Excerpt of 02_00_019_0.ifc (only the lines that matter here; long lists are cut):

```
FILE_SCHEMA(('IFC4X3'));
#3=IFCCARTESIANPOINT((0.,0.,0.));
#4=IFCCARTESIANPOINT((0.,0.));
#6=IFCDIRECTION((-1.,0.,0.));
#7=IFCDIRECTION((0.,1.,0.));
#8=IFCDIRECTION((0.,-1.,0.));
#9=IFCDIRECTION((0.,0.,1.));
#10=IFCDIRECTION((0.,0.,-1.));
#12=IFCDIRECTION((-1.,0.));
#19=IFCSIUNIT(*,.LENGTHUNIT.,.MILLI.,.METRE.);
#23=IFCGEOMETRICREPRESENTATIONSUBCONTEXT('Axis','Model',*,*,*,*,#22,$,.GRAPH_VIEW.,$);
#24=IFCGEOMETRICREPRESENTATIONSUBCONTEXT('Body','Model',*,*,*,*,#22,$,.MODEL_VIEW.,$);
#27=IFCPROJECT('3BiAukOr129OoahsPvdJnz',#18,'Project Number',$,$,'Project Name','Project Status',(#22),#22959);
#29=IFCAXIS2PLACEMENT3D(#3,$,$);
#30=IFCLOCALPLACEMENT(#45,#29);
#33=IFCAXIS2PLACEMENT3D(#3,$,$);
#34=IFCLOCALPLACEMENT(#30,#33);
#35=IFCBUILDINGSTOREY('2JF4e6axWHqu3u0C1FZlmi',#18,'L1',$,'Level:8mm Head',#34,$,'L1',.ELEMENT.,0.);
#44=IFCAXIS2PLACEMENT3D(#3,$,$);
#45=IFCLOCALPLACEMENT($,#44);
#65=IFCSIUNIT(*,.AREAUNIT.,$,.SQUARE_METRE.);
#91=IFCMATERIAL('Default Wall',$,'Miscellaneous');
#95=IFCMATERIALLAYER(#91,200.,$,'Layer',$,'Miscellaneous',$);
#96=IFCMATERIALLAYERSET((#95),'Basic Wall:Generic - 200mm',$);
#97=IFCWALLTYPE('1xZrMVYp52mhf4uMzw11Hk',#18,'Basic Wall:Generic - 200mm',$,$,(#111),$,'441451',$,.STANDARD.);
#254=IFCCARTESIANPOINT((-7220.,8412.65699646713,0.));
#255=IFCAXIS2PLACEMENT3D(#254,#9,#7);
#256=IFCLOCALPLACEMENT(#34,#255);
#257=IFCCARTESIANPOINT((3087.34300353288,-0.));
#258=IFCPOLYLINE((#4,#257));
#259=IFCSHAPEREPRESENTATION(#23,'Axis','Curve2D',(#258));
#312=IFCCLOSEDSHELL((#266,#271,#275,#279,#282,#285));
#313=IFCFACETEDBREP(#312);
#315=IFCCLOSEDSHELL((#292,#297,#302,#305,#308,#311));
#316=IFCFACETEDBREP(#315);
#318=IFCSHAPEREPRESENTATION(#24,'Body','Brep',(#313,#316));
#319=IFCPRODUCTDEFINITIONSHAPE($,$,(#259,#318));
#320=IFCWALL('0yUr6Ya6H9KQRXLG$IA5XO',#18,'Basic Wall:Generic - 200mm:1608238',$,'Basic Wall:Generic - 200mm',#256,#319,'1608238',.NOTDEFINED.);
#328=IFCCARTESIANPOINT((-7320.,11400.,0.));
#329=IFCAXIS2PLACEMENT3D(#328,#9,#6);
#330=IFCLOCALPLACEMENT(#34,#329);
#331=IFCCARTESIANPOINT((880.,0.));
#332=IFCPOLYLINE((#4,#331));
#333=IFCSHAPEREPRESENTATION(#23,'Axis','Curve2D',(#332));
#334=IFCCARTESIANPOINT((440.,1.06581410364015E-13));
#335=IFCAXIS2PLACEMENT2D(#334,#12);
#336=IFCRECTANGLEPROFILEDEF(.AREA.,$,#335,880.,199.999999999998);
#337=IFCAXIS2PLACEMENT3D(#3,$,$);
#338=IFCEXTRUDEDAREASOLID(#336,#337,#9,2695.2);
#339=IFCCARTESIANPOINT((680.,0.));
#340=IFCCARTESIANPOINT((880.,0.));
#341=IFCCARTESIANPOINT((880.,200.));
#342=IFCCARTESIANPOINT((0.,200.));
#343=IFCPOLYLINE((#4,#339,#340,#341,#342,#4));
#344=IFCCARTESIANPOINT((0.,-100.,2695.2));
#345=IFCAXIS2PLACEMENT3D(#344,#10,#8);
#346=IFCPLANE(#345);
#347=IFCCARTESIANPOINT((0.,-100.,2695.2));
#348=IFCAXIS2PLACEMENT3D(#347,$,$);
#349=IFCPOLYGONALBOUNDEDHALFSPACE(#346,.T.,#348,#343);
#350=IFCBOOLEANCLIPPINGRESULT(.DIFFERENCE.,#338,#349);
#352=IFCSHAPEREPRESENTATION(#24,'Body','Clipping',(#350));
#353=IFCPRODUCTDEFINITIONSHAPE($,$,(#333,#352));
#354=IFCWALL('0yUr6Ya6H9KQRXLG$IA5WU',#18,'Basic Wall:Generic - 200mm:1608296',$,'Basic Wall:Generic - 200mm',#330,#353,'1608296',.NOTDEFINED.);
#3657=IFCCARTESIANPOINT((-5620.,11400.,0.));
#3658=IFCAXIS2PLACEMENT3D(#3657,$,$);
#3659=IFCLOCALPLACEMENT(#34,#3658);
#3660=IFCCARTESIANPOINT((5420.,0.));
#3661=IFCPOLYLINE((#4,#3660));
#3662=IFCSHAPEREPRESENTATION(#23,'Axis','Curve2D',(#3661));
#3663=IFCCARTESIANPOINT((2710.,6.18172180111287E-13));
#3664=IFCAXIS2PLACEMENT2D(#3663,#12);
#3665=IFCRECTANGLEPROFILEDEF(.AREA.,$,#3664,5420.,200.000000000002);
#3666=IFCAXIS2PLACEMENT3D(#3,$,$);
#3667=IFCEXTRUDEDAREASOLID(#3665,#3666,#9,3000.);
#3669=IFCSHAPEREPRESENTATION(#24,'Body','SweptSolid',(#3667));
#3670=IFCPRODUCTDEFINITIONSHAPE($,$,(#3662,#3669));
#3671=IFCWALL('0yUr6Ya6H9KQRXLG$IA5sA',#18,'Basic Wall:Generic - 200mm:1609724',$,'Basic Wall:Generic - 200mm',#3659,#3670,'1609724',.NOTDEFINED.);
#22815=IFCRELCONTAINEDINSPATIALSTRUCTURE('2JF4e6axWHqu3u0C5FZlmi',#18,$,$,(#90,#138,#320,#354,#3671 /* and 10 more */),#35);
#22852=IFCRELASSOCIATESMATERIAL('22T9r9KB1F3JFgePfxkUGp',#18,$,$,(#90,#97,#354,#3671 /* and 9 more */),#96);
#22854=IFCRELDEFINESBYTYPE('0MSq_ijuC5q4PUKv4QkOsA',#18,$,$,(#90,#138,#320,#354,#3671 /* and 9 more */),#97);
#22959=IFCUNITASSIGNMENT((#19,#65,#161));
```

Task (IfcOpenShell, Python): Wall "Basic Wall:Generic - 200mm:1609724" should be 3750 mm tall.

```python
import ifcopenshell
import ifcopenshell.geom
import ifcopenshell.util.representation
import ifcopenshell.util.shape
import ifcopenshell.util.unit

model = ifcopenshell.open("02_00_019_0.ifc")
unit_scale = ifcopenshell.util.unit.calculate_unit_scale(model)
settings = ifcopenshell.geom.settings()


def volume(element):
    """Net volume in cubic metres, openings subtracted."""
    shape = ifcopenshell.geom.create_shape(settings, element)
    return ifcopenshell.util.shape.get_volume(shape.geometry)


wall = model.by_guid("0yUr6Ya6H9KQRXLG$IA5sA")
before = volume(wall)

body = ifcopenshell.util.representation.get_representation(wall, "Model", "Body")
solid = body.Items[0]
old_height = solid.Depth
solid.Depth = 3.75 / unit_scale
after = volume(wall)

print(f"height {old_height:g} -> {solid.Depth:g}, volume {before:.3f} -> {after:.3f} m3")

model.write("02_00_019_0_rev.ifc")
```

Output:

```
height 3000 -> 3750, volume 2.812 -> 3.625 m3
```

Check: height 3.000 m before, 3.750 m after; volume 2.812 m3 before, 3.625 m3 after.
